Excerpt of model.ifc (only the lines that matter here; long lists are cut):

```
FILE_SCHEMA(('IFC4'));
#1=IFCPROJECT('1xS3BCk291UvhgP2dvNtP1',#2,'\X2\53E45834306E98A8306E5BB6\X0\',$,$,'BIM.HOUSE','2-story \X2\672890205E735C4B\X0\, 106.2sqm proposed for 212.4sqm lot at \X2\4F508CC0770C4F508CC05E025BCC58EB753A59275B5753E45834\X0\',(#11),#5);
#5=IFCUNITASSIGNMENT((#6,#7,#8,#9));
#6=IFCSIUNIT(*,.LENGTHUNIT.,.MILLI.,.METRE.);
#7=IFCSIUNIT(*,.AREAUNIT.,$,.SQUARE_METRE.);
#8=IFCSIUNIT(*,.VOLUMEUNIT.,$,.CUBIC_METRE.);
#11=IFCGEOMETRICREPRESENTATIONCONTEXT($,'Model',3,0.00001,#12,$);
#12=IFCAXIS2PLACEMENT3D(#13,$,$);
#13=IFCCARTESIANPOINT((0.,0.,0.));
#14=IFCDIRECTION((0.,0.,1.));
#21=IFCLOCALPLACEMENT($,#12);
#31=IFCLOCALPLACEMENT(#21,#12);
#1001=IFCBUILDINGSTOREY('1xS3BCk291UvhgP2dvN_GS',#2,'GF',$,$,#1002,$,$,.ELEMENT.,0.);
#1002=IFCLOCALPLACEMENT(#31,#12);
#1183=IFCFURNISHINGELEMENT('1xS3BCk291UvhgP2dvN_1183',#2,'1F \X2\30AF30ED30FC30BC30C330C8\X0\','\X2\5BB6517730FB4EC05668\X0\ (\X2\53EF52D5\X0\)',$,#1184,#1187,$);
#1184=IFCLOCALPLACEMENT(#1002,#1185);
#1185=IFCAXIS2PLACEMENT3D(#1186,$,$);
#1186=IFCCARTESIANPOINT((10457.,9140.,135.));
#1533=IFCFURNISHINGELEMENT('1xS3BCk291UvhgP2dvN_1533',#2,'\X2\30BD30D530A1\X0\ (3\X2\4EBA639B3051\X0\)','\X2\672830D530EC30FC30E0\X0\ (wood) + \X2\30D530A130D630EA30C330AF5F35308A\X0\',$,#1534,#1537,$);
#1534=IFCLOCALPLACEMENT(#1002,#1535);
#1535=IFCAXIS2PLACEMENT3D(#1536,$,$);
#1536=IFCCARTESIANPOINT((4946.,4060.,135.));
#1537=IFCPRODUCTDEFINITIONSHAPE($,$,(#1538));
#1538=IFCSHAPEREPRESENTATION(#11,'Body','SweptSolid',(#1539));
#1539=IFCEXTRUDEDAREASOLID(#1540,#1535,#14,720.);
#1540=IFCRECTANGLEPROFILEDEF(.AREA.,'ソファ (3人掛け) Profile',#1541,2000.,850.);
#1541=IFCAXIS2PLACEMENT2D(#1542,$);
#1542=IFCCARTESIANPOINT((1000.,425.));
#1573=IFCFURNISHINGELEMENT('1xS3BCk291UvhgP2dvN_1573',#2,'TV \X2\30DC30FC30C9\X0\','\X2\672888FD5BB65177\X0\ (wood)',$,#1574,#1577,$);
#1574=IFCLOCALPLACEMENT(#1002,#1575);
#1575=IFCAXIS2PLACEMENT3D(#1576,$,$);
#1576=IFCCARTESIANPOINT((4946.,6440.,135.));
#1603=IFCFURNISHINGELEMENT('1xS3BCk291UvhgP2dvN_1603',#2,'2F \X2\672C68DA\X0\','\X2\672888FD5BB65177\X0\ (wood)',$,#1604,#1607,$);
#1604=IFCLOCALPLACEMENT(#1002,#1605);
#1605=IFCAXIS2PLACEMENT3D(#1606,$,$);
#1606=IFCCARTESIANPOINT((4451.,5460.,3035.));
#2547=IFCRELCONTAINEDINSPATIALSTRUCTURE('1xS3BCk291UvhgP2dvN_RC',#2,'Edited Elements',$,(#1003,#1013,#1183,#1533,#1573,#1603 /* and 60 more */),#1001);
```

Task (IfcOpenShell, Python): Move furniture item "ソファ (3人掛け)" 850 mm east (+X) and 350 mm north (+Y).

```python
import ifcopenshell
import ifcopenshell.api.geometry
import ifcopenshell.util.placement
import ifcopenshell.util.unit

model = ifcopenshell.open("model.ifc")
unit_scale = ifcopenshell.util.unit.calculate_unit_scale(model)

item = model.by_id(1533)
matrix = ifcopenshell.util.placement.get_local_placement(item.ObjectPlacement)
matrix[0, 3] += 0.85 / unit_scale
matrix[1, 3] += 0.35 / unit_scale
ifcopenshell.api.geometry.edit_object_placement(model, product=item, matrix=matrix, is_si=False)

print(ifcopenshell.util.placement.get_local_placement(item.ObjectPlacement).round(3) + 0.0)

model.write("model_edited.ifc")
```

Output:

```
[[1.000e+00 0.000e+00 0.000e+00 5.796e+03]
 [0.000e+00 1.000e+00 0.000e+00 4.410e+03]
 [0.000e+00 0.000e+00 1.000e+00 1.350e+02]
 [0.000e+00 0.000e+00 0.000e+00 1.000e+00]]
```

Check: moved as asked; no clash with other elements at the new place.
